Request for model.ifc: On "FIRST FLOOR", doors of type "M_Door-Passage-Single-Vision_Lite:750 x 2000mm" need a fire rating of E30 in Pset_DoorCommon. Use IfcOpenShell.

First a look at what the model holds.

```python
import ifcopenshell
import ifcopenshell.util.element

model = ifcopenshell.open("model.ifc")
print(model.schema)
storey = next(s for s in model.by_type("IfcBuildingStorey") if s.Name == "FIRST FLOOR")
doors = [e for e in ifcopenshell.util.element.get_decomposition(storey) if e.is_a("IfcDoor")]
seen = {}
for e in doors:
    element_type = ifcopenshell.util.element.get_type(e)
    key = (element_type.Name if element_type != e and element_type else None, ifcopenshell.util.element.get_pset(e, "Pset_DoorCommon", "FireRating"))
    seen[key] = seen.get(key, 0) + 1
for (name, value), count in sorted(seen.items(), key=str):
    print(count, "x", name, "|", value)
```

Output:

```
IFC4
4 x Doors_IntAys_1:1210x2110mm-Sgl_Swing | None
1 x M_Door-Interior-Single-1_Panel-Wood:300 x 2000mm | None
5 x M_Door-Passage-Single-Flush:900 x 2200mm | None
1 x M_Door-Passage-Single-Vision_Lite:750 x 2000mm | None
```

```python
import ifcopenshell
import ifcopenshell.api.pset
import ifcopenshell.util.element

model = ifcopenshell.open("model.ifc")

storey = next(s for s in model.by_type("IfcBuildingStorey") if s.Name == "FIRST FLOOR")
doors = [e for e in ifcopenshell.util.element.get_decomposition(storey) if e.is_a("IfcDoor")]

count = 0
for e in doors:
    element_type = ifcopenshell.util.element.get_type(e)
    if element_type in (None, e) or element_type.Name != "M_Door-Passage-Single-Vision_Lite:750 x 2000mm":
        continue
    # add_pset returns the element's existing set when there is one.
    pset = ifcopenshell.api.pset.add_pset(model, product=e, name="Pset_DoorCommon")
    ifcopenshell.api.pset.edit_pset(model, pset=pset, properties={"FireRating": "E30"})
    count += 1

print(count, "doors updated")

model.write("model_updated.ifc")
```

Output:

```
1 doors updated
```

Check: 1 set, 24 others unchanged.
